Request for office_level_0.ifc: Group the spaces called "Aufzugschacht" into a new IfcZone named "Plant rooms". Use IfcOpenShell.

First a look at what the model holds.

```python
import ifcopenshell

model = ifcopenshell.open("office_level_0.ifc")
print(model.schema)
seen = {}
for space in model.by_type("IfcSpace"):
    seen[space.LongName] = seen.get(space.LongName, 0) + 1
for name, count in sorted(seen.items(), key=str):
    print(count, "x", name)
print("zones:", [z.Name for z in model.by_type("IfcZone")][:20])
```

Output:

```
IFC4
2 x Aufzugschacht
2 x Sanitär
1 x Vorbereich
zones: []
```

```python
import ifcopenshell
import ifcopenshell.api.group
import ifcopenshell.api.root

model = ifcopenshell.open("office_level_0.ifc")

names = {"Aufzugschacht"}
spaces = [s for s in model.by_type("IfcSpace") if s.LongName in names]

zone = ifcopenshell.api.root.create_entity(model, ifc_class="IfcZone", name="Plant rooms")
ifcopenshell.api.group.assign_group(model, products=spaces, group=zone)
print(len(spaces), "spaces in", zone.Name)

model.write("office_level_0_updated.ifc")
```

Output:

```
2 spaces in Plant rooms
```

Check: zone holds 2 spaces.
